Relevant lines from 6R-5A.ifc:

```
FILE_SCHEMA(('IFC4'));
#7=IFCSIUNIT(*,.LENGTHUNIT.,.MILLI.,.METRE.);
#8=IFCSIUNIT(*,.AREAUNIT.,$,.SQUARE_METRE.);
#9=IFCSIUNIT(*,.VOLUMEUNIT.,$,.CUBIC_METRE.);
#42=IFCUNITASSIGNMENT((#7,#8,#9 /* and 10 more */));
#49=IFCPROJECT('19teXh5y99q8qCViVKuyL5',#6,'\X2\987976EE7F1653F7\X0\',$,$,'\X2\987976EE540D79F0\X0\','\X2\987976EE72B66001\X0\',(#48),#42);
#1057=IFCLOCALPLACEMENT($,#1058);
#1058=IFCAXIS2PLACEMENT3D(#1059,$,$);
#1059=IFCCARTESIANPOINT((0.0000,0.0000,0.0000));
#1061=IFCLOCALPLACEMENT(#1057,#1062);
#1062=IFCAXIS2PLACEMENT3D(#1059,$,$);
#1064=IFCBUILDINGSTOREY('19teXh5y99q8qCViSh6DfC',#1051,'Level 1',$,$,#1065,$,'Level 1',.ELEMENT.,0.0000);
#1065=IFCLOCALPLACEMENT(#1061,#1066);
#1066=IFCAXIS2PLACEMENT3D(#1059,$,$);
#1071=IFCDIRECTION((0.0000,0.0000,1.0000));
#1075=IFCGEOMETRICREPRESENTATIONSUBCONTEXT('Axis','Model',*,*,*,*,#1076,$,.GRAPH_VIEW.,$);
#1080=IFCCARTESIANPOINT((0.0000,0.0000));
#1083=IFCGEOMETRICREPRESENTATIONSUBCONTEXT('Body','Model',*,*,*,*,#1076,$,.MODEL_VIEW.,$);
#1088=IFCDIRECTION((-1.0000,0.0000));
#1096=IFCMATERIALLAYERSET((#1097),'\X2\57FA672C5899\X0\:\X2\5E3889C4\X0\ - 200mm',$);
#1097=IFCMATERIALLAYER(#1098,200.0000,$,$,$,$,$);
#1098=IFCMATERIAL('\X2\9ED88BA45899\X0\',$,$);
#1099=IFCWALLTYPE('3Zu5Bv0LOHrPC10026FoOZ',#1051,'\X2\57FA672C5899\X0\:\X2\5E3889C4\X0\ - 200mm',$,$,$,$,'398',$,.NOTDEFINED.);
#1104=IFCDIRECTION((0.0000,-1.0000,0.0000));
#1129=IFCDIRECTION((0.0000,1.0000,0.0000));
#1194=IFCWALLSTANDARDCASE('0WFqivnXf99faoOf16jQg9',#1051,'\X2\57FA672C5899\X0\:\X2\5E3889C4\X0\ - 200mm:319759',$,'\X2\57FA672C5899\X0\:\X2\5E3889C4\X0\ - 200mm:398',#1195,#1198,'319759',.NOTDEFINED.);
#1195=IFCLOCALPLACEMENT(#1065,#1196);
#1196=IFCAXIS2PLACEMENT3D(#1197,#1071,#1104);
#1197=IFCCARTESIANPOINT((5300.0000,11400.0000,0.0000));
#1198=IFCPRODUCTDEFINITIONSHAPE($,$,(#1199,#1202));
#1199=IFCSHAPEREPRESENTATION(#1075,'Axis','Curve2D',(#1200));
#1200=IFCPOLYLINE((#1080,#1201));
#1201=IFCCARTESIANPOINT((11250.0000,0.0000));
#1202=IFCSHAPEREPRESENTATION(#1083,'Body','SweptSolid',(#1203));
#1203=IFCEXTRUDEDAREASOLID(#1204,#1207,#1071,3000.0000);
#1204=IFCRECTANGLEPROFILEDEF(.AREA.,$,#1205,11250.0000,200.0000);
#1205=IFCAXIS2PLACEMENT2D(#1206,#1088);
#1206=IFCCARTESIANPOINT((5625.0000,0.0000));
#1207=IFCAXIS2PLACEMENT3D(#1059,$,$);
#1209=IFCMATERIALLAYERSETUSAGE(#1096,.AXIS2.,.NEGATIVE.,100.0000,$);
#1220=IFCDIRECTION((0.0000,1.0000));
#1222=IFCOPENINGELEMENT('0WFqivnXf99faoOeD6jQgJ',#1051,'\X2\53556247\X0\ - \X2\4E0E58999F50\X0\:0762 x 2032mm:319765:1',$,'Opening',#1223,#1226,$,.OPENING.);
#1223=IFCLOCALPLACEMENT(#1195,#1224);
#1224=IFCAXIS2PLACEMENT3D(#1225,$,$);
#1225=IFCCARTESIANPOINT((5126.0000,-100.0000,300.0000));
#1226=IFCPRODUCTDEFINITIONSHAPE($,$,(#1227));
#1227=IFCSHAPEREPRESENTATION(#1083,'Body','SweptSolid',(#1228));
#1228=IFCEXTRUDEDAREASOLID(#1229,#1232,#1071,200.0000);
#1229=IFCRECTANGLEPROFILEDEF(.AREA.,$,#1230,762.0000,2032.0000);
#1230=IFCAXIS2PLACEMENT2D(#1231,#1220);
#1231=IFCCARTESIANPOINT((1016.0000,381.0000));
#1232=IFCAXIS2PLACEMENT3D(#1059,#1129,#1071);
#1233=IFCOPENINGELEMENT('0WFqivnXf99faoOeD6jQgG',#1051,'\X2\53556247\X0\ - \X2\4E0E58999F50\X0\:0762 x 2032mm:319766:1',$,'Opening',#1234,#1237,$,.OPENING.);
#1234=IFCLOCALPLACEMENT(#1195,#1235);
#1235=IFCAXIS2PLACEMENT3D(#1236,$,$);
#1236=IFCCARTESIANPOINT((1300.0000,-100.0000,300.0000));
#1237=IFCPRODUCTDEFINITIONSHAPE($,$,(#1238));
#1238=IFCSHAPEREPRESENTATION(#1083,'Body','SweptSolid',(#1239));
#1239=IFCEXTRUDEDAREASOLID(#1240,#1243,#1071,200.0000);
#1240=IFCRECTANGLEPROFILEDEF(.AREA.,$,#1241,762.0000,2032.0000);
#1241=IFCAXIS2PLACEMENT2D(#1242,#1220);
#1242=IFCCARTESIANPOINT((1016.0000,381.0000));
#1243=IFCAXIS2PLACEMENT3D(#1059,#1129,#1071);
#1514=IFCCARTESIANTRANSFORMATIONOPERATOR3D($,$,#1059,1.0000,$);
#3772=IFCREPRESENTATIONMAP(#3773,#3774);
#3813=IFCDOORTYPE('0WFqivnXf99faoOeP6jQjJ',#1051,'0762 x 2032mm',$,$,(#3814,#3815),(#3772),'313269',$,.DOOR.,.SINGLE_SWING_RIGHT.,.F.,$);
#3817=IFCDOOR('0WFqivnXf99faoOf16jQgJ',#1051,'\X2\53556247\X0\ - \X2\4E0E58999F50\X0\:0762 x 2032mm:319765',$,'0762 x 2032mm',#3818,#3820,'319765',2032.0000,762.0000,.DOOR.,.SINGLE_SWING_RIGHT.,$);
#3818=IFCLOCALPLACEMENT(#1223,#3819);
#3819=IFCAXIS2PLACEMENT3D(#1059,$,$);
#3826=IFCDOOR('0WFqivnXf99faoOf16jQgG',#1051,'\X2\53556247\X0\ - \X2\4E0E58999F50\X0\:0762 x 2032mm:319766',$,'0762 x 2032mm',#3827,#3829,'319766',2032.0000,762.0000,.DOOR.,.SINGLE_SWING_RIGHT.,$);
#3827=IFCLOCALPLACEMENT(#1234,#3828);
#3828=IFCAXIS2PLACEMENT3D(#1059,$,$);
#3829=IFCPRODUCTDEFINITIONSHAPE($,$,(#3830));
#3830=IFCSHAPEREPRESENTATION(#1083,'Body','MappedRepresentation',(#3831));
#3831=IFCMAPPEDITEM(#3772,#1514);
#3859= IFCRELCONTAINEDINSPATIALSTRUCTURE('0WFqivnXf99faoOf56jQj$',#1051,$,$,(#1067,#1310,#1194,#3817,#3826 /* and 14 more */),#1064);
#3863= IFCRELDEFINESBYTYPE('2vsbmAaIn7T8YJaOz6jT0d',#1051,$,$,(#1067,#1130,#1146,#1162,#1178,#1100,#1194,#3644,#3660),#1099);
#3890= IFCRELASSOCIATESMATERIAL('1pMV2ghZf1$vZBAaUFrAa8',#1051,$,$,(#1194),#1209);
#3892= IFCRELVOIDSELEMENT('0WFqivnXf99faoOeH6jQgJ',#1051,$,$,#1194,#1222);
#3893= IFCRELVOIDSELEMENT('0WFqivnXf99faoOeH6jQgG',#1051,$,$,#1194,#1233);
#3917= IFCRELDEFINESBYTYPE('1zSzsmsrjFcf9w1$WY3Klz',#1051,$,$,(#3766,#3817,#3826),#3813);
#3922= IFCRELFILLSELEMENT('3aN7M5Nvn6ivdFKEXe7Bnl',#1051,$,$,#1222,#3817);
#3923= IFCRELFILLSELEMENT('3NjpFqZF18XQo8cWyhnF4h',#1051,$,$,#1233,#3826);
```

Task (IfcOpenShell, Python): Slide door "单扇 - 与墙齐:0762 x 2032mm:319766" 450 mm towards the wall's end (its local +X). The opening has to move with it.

```python
import ifcopenshell
import ifcopenshell.api.geometry
import ifcopenshell.util.placement
import ifcopenshell.util.unit

model = ifcopenshell.open("6R-5A.ifc")
unit_scale = ifcopenshell.util.unit.calculate_unit_scale(model)

door = model.by_id(3826)
opening = door.FillsVoids[0].RelatingOpeningElement
wall = opening.VoidsElements[0].RelatingBuildingElement

wall_matrix = ifcopenshell.util.placement.get_local_placement(wall.ObjectPlacement)
shift = wall_matrix[:3, 0] * 0.45 / unit_scale
before = ifcopenshell.util.placement.get_local_placement(door.ObjectPlacement)[:3, 3].copy()

# The door is placed relative to its opening, so it follows when the opening moves.
matrix = ifcopenshell.util.placement.get_local_placement(opening.ObjectPlacement)
matrix[:3, 3] += shift
ifcopenshell.api.geometry.edit_object_placement(
    model, product=opening, matrix=matrix, is_si=False, should_transform_children=True
)

after = ifcopenshell.util.placement.get_local_placement(door.ObjectPlacement)[:3, 3]
print("door moved by", (after - before).round(3) + 0.0)

model.write("6R-5A_edited.ifc")
```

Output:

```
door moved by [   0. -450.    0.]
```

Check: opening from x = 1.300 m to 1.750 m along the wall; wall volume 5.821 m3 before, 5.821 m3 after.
